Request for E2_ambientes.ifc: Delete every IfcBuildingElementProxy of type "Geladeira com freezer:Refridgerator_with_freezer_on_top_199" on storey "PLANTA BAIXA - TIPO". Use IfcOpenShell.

First a look at what the model holds.

```python
import ifcopenshell
import ifcopenshell.util.element

model = ifcopenshell.open("E2_ambientes.ifc")
print(model.schema)
storey = next(s for s in model.by_type("IfcBuildingStorey") if s.Name == "PLANTA BAIXA - TIPO")
proxies = [e for e in ifcopenshell.util.element.get_decomposition(storey) if e.is_a("IfcBuildingElementProxy")]
seen = {}
for e in proxies:
    element_type = ifcopenshell.util.element.get_type(e)
    name = element_type.Name if element_type not in (None, e) else None
    seen[name] = seen.get(name, 0) + 1
for name, count in sorted(seen.items(), key=str):
    print(count, "x", name)
```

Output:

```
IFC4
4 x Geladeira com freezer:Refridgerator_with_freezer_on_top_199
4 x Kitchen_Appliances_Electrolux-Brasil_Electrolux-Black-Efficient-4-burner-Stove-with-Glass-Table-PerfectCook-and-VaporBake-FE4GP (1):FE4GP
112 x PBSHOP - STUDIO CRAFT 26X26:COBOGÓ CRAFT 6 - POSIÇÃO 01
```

```python
import ifcopenshell
import ifcopenshell.api.root
import ifcopenshell.util.element

model = ifcopenshell.open("E2_ambientes.ifc")

storey = next(s for s in model.by_type("IfcBuildingStorey") if s.Name == "PLANTA BAIXA - TIPO")
proxies = [e for e in ifcopenshell.util.element.get_decomposition(storey) if e.is_a("IfcBuildingElementProxy")]
targets = [e for e in proxies if (t := ifcopenshell.util.element.get_type(e)) not in (None, e) and t.Name == "Geladeira com freezer:Refridgerator_with_freezer_on_top_199"]

for e in targets:
    ifcopenshell.api.root.remove_product(model, product=e)
print(len(targets), "removed")

model.write("E2_ambientes_rev.ifc")
```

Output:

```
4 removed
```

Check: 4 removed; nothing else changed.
